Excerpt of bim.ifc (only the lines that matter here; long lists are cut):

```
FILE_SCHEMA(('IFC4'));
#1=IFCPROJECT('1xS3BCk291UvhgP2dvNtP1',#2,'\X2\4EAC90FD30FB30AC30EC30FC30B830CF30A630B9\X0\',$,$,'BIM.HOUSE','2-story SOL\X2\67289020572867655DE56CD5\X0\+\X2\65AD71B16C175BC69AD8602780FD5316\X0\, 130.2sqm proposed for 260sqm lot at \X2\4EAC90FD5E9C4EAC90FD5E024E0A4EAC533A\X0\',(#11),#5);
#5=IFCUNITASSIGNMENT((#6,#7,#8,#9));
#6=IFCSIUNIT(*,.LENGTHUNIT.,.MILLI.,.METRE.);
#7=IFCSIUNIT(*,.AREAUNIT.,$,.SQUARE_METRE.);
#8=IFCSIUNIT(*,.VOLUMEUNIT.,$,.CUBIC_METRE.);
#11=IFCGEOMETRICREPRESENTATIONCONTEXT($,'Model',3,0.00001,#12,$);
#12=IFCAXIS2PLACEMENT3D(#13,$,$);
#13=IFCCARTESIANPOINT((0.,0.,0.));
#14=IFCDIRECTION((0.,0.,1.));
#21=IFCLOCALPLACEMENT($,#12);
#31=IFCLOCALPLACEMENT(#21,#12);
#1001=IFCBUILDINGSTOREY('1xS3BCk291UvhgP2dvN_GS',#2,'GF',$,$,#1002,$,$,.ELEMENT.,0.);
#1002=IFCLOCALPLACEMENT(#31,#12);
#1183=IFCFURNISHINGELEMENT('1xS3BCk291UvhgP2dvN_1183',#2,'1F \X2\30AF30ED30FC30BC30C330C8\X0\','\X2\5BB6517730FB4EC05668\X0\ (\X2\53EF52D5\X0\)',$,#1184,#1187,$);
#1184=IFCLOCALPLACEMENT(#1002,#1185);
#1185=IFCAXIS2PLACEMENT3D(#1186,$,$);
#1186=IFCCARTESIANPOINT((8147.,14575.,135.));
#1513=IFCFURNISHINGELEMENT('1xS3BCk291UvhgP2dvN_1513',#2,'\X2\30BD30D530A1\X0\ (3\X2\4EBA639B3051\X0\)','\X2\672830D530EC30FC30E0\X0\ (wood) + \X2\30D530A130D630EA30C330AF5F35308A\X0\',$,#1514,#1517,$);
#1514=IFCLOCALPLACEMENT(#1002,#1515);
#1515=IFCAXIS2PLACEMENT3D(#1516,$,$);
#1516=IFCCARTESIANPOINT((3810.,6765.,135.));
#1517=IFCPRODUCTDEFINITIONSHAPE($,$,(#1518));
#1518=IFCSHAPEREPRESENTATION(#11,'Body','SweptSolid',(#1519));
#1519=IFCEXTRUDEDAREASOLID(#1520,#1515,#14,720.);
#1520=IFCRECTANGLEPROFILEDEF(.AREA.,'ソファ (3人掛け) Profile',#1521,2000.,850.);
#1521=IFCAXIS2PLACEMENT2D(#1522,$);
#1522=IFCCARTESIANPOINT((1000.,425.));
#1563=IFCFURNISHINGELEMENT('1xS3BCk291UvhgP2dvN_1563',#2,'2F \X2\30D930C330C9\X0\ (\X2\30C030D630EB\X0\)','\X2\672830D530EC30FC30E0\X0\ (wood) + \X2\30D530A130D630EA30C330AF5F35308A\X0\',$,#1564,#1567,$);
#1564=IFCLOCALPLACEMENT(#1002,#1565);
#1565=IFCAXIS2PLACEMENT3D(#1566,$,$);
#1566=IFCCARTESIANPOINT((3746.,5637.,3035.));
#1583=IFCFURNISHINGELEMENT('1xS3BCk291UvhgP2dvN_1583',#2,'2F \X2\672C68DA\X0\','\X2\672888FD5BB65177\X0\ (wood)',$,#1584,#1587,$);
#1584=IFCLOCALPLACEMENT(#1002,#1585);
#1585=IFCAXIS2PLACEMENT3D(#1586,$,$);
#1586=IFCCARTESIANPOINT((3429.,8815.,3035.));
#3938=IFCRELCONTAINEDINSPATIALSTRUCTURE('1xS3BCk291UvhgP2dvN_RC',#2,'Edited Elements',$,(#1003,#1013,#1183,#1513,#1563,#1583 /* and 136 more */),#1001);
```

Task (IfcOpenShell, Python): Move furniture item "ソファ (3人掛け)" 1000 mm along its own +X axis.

```python
import ifcopenshell
import ifcopenshell.api.geometry
import ifcopenshell.util.placement
import ifcopenshell.util.unit

model = ifcopenshell.open("bim.ifc")
unit_scale = ifcopenshell.util.unit.calculate_unit_scale(model)

item = model.by_id(1513)
matrix = ifcopenshell.util.placement.get_local_placement(item.ObjectPlacement)
matrix[:3, 3] += matrix[:3, 0] * 1 / unit_scale
ifcopenshell.api.geometry.edit_object_placement(model, product=item, matrix=matrix, is_si=False)

print(ifcopenshell.util.placement.get_local_placement(item.ObjectPlacement).round(3) + 0.0)

model.write("bim_edited.ifc")
```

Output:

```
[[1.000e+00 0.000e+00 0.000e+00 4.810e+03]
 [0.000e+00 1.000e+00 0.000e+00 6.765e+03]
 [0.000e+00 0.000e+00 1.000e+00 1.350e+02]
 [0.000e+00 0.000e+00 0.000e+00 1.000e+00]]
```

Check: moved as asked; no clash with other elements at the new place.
